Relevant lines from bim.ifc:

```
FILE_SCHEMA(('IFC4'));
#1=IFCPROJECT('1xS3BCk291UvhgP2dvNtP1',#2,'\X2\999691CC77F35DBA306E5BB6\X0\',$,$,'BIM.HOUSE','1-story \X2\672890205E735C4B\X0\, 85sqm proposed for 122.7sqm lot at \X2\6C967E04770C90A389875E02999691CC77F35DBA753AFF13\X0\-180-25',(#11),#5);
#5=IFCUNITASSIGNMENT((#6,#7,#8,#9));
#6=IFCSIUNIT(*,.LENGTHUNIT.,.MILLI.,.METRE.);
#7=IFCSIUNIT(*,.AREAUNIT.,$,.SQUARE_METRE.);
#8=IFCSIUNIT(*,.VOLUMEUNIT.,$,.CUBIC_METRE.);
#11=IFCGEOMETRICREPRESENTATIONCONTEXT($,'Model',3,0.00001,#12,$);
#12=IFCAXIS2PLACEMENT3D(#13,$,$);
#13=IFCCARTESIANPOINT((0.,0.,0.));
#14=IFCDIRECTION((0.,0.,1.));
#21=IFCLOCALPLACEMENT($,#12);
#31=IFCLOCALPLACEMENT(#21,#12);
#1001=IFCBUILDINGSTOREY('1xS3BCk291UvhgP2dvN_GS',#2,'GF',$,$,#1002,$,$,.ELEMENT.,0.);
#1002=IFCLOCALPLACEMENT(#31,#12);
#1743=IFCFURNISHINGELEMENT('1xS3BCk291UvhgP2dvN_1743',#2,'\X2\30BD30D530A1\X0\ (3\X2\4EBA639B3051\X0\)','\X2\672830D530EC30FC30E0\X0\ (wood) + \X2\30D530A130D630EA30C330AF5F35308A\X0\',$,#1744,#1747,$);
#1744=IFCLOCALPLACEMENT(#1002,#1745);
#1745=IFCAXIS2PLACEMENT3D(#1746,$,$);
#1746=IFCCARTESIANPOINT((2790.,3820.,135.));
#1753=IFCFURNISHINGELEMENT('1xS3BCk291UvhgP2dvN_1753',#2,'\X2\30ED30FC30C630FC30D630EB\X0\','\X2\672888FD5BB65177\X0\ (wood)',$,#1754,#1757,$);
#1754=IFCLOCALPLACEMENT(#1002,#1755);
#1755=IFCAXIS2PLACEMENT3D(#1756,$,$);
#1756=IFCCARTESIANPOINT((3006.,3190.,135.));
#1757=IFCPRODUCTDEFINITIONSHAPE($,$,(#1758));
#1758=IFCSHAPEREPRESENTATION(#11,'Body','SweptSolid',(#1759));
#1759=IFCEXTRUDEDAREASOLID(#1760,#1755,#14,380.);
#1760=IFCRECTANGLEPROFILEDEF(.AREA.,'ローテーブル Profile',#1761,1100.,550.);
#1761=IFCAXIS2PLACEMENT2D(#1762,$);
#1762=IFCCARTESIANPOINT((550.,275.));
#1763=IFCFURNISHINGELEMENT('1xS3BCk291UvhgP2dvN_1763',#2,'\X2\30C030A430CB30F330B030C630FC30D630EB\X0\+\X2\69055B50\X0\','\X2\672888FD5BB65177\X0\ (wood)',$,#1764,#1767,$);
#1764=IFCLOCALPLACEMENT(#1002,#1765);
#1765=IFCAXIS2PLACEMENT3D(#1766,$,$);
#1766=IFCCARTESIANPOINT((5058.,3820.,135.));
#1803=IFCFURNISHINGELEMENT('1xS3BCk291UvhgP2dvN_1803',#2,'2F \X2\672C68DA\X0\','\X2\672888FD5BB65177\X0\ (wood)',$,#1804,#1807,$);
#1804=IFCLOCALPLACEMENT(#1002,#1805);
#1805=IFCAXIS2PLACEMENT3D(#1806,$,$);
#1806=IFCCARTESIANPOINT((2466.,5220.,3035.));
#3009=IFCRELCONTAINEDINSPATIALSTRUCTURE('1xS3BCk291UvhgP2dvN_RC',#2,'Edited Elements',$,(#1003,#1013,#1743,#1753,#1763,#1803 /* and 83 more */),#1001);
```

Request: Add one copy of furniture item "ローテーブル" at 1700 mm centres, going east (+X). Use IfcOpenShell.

```python
import numpy as np
import ifcopenshell
import ifcopenshell.api.geometry
import ifcopenshell.api.root
import ifcopenshell.util.element
import ifcopenshell.util.placement

model = ifcopenshell.open("bim.ifc")


def reuse_history(source, copy):
    """copy_class also copies each property set's owner history, people and application; keep the originals."""
    for rel in copy.IsDefinedBy:
        if rel.is_a("IfcRelDefinesByProperties") and (history := rel.RelatingPropertyDefinition.OwnerHistory):
            rel.RelatingPropertyDefinition.OwnerHistory = source.OwnerHistory
            ifcopenshell.util.element.remove_deep2(model, history)


source = model.by_id(1753)
base = ifcopenshell.util.placement.get_local_placement(source.ObjectPlacement)
step = np.array([1.0, 0.0, 0.0]) * 1700.0

for i in range(1, 2):
    copy = ifcopenshell.api.root.copy_class(model, product=source)
    copy.Representation = ifcopenshell.util.element.copy_deep(
        model, source.Representation, exclude=["IfcGeometricRepresentationContext", "IfcRepresentationMap"]
    )
    reuse_history(source, copy)
    matrix = base.copy()
    matrix[:3, 3] += i * step
    print("added at", matrix[:3, 3].round(3) + 0.0)
    ifcopenshell.api.geometry.edit_object_placement(model, product=copy, matrix=matrix, is_si=False)

model.write("bim-out.ifc")
```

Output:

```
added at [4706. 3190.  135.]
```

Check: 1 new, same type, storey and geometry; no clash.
